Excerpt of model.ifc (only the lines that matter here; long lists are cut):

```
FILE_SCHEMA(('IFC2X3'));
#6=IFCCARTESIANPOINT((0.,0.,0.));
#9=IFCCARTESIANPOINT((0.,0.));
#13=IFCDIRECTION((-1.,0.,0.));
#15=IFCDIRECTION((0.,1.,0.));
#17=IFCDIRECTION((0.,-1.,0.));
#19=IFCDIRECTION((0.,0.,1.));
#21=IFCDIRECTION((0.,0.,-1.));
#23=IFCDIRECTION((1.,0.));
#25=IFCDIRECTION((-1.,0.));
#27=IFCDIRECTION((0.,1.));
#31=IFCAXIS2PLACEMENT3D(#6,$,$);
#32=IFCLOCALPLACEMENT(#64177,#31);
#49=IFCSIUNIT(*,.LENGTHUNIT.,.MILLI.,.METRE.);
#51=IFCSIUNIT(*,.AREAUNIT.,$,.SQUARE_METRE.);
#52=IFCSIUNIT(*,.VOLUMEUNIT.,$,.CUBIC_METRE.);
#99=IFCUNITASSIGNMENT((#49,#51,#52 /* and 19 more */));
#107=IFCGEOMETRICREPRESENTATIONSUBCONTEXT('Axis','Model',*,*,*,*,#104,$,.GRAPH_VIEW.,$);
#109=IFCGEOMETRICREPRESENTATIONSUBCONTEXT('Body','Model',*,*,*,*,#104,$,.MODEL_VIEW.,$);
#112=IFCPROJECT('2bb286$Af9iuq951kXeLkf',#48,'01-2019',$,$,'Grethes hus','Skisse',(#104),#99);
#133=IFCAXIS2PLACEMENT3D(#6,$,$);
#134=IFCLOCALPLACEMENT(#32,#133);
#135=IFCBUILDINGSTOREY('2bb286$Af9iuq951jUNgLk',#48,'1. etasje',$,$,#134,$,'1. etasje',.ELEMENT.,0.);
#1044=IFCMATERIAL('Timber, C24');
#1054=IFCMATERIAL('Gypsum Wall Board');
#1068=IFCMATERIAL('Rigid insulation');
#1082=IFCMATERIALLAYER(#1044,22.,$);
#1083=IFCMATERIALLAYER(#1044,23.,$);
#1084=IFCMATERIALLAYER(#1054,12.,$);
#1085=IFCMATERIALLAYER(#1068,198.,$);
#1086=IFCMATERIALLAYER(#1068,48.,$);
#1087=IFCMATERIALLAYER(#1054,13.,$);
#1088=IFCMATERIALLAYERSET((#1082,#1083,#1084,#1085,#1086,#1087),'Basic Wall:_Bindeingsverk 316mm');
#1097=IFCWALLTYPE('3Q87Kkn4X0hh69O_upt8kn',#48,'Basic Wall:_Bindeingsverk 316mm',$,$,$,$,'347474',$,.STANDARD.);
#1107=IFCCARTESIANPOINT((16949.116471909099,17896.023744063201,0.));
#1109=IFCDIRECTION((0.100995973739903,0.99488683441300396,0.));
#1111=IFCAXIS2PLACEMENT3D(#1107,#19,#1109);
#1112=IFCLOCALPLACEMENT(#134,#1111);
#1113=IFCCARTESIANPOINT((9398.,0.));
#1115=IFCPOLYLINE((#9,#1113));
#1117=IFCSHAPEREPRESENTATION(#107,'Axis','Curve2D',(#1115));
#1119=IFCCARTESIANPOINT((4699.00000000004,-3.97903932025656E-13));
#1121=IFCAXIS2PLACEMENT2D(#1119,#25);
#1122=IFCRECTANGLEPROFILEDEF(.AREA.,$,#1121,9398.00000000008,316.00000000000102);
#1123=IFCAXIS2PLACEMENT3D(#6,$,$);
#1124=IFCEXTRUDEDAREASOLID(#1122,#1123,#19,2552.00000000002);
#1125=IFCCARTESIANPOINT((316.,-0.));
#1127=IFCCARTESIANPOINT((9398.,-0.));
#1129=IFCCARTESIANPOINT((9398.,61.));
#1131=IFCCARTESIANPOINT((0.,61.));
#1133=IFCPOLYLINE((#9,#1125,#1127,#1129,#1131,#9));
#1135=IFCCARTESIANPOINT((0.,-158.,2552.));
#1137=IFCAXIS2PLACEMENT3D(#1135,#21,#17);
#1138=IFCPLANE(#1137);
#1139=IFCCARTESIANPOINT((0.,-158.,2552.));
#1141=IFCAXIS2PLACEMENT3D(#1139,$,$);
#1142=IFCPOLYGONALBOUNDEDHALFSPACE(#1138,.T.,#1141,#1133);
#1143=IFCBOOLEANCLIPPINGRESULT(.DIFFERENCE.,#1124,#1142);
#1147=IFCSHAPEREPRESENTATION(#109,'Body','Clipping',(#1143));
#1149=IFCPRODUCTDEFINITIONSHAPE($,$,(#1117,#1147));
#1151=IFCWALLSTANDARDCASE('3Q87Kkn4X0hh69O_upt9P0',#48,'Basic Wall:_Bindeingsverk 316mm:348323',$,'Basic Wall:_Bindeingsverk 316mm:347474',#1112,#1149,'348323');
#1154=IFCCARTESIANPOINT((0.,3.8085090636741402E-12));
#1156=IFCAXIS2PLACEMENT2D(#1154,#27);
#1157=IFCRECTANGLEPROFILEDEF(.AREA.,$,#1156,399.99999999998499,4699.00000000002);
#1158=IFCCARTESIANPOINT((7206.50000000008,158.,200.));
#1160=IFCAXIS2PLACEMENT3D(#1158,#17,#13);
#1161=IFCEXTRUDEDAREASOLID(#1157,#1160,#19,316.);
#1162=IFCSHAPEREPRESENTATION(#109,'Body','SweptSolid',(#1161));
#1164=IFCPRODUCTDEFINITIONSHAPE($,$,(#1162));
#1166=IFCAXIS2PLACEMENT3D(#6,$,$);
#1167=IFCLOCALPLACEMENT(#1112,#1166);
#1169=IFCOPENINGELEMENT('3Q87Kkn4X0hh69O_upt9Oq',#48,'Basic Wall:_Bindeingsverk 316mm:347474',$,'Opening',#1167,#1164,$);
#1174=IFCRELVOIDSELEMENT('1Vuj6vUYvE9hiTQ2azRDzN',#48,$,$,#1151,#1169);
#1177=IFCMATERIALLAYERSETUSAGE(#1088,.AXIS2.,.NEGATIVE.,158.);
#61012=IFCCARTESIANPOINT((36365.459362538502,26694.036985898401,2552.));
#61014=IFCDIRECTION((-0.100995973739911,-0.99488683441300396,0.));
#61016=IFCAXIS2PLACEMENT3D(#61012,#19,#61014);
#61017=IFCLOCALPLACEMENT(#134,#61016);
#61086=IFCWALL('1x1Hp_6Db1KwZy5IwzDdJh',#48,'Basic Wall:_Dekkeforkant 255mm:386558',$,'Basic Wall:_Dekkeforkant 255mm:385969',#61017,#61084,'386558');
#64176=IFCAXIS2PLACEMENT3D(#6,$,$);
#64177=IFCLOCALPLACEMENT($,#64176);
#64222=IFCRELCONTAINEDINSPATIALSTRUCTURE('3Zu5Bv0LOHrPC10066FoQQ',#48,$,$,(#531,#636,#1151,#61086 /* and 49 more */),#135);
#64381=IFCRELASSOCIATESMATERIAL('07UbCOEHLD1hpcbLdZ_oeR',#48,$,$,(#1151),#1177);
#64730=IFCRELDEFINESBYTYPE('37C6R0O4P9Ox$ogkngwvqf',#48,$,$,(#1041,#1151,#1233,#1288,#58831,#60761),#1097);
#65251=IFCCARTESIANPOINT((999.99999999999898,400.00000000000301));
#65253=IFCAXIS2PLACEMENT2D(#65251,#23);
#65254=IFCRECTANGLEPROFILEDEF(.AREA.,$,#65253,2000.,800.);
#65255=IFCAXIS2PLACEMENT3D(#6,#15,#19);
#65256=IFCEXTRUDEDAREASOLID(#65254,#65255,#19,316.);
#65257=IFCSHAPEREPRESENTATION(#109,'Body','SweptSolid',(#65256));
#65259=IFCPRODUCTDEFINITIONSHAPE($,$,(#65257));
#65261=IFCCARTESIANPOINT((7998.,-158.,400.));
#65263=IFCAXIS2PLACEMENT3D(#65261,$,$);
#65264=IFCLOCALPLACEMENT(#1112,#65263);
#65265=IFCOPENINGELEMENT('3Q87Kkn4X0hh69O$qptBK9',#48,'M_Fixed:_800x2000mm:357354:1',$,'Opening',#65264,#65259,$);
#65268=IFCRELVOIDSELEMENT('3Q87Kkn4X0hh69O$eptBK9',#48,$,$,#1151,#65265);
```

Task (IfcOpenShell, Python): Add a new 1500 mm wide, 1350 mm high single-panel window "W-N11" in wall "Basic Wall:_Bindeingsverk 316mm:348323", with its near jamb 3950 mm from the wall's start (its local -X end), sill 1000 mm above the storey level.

```python
import numpy as np
import ifcopenshell
import ifcopenshell.api.feature
import ifcopenshell.api.geometry
import ifcopenshell.api.root
import ifcopenshell.api.spatial
import ifcopenshell.api.type
import ifcopenshell.geom
import ifcopenshell.util.element
import ifcopenshell.util.placement
import ifcopenshell.util.representation
import ifcopenshell.util.shape
import ifcopenshell.util.unit

model = ifcopenshell.open("model.ifc")
unit_scale = ifcopenshell.util.unit.calculate_unit_scale(model)
settings = ifcopenshell.geom.settings()


def volume(element):
    """Net volume in cubic metres, openings subtracted."""
    shape = ifcopenshell.geom.create_shape(settings, element)
    return ifcopenshell.util.shape.get_volume(shape.geometry)


wall = model.by_guid("3Q87Kkn4X0hh69O_upt9P0")
storey = ifcopenshell.util.element.get_container(wall, ifc_class="IfcBuildingStorey")
context = ifcopenshell.util.representation.get_context(model, "Model", "Body", "MODEL_VIEW")
before = volume(wall)

width, height, from_end, sill = 1.5, 1.35, 3.95, 1  # metres

# The wall runs along its own X axis, and the end named is its -X end.
wall_shape = ifcopenshell.geom.create_shape(settings, wall)
x, y, z = ifcopenshell.util.shape.get_vertices(wall_shape.geometry).T
start = x.min() + from_end
face, thickness = float(y.min()), float(y.max() - y.min())
wall_matrix = ifcopenshell.util.placement.get_local_placement(wall.ObjectPlacement)
level = ifcopenshell.util.placement.get_local_placement(storey.ObjectPlacement)[2, 3]


def in_wall(x, y):
    """Placement at x, y metres in the wall's axes, at sill height."""
    matrix = wall_matrix.copy()
    matrix[:, 3] = wall_matrix @ np.array([x / unit_scale, y / unit_scale, 0.0, 1.0])
    matrix[2, 3] = level + sill / unit_scale
    return matrix


# Opening: a box that overshoots both wall faces by 50 mm.
opening = ifcopenshell.api.root.create_entity(model, ifc_class="IfcOpeningElement")
box = ifcopenshell.api.geometry.add_wall_representation(
    model, context=context, length=width, height=height, thickness=thickness + 0.1
)
ifcopenshell.api.geometry.assign_representation(model, product=opening, representation=box)
ifcopenshell.api.geometry.edit_object_placement(model, product=opening, matrix=in_wall(start, face - 0.05), is_si=False)
ifcopenshell.api.feature.add_feature(model, feature=opening, element=wall)

window = ifcopenshell.api.root.create_entity(model, ifc_class="IfcWindow", name="W-N11")
window.OverallWidth, window.OverallHeight = width / unit_scale, height / unit_scale
body = ifcopenshell.api.geometry.add_window_representation(
    model,
    context=context,
    overall_width=window.OverallWidth,
    overall_height=window.OverallHeight,
    partition_type="SINGLE_PANEL",
)
ifcopenshell.api.geometry.assign_representation(model, product=window, representation=body)
ifcopenshell.api.spatial.assign_container(model, products=[window], relating_structure=storey)
fills = ifcopenshell.api.feature.add_filling(model, opening=opening, element=window)
fills.OwnerHistory = window.OwnerHistory  # required in IFC2X3

# IFC2X3 keeps the operation on the window style.
style = ifcopenshell.api.root.create_entity(model, ifc_class="IfcWindowStyle", name="W-N11")
style.OperationType, style.ConstructionType = "SINGLE_PANEL", "NOTDEFINED"
style.ParameterTakesPrecedence = style.Sizeable = False
ifcopenshell.api.type.assign_type(model, related_objects=[window], relating_type=style)

# Centre the window in the wall's thickness.
ifcopenshell.api.geometry.edit_object_placement(model, product=window, matrix=in_wall(start, face), is_si=False)
window_shape = ifcopenshell.geom.create_shape(settings, window)
depth = ifcopenshell.util.shape.get_vertices(window_shape.geometry)[:, 1]
offset = face + thickness / 2 - (depth.min() + depth.max()) / 2
ifcopenshell.api.geometry.edit_object_placement(model, product=window, matrix=in_wall(start, offset), is_si=False)

after = volume(wall)

print(f"wall volume {before:.3f} -> {after:.3f} m3")

model.write("model-out.ifc")
```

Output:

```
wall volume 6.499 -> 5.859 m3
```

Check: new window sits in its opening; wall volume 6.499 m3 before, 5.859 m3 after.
